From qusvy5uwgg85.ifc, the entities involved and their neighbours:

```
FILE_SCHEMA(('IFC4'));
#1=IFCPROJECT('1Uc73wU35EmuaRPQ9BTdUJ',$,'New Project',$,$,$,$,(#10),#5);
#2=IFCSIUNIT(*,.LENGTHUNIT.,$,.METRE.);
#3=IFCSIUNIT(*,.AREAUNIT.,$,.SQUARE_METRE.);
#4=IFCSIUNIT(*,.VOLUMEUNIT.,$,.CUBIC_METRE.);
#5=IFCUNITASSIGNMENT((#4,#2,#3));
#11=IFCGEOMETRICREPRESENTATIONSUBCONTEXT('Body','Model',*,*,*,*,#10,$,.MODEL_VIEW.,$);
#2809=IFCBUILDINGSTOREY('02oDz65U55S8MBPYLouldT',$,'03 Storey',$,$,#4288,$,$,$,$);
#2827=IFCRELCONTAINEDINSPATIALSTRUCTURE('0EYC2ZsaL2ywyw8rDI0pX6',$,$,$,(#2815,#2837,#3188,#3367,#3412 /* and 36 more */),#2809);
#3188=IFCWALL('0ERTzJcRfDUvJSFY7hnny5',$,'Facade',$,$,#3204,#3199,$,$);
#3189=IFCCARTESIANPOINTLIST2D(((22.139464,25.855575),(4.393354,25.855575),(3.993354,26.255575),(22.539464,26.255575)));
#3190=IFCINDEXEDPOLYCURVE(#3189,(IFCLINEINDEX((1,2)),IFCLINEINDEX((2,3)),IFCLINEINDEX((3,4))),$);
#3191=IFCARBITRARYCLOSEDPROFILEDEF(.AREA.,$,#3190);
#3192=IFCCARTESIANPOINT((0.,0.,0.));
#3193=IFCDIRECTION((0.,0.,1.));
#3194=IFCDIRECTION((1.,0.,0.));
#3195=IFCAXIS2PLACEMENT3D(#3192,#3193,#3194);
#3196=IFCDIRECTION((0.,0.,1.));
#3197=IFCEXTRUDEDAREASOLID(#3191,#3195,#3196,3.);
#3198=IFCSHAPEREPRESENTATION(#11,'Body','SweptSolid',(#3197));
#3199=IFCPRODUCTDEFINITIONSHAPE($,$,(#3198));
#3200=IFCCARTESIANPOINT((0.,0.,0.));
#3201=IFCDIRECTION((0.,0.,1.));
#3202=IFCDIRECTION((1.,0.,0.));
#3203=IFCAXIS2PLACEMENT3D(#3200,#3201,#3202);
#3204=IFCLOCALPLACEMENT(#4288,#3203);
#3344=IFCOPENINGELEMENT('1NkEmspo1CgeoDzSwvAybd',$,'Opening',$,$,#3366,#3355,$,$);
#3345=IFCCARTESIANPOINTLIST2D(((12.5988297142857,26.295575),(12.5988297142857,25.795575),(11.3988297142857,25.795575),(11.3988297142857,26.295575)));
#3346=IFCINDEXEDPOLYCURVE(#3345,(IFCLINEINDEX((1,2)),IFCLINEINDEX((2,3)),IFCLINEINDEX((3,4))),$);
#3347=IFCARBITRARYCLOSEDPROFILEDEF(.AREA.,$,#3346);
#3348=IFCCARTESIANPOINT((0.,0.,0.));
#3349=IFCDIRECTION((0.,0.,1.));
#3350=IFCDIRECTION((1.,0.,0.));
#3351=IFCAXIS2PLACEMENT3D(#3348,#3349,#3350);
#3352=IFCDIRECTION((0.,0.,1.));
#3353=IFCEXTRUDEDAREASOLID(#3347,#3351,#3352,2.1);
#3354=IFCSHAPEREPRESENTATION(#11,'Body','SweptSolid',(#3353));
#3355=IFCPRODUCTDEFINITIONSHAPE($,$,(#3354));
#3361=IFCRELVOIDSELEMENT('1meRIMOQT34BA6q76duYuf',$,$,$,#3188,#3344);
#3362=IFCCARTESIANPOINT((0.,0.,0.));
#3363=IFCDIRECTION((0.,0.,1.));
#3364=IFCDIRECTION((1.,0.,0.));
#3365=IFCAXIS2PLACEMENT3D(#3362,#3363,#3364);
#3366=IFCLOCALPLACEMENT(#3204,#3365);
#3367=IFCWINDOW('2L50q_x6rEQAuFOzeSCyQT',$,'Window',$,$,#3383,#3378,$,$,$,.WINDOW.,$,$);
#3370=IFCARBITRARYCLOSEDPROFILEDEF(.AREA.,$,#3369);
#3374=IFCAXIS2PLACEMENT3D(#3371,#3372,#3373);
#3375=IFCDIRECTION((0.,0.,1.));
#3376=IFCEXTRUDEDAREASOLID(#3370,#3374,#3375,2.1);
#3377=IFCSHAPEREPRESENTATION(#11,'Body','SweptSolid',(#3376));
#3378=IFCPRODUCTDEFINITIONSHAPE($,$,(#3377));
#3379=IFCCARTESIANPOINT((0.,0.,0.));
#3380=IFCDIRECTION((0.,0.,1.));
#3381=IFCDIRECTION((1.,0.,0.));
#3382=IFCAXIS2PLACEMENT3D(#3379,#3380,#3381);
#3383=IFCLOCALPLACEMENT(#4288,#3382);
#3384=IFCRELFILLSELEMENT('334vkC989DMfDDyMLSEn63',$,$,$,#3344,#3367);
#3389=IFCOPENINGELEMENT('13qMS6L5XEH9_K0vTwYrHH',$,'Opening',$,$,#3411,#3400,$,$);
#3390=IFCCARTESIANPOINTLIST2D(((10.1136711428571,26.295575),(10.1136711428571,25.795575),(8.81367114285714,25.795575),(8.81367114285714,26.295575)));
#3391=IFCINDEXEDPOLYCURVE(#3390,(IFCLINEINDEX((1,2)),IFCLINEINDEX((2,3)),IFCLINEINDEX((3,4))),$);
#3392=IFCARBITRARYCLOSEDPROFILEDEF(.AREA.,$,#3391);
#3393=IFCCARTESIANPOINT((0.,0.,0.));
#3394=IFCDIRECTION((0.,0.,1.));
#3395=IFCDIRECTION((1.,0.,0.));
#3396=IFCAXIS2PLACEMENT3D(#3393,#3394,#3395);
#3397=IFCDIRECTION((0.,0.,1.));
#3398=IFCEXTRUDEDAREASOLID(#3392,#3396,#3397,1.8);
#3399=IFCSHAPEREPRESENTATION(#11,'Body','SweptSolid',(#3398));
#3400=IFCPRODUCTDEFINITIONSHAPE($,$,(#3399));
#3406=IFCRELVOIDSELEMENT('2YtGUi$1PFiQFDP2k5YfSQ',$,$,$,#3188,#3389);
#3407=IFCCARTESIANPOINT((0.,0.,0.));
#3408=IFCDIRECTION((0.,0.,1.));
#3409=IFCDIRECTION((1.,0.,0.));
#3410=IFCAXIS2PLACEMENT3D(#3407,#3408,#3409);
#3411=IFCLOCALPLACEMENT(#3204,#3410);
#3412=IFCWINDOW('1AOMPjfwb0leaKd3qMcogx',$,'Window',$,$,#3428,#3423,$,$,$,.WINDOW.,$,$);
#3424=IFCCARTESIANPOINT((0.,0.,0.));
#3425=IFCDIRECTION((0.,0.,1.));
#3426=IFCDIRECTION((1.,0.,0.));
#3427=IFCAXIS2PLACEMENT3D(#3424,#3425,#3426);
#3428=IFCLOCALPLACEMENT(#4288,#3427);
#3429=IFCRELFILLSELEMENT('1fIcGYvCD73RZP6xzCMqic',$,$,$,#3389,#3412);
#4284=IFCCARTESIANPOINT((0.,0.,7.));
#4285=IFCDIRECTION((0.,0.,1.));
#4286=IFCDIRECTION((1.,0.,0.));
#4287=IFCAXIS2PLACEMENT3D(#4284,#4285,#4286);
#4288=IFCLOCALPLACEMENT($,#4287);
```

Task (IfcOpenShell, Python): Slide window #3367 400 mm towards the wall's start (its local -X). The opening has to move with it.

```python
import ifcopenshell
import ifcopenshell.api.geometry
import ifcopenshell.util.placement
import ifcopenshell.util.unit

model = ifcopenshell.open("qusvy5uwgg85.ifc")
unit_scale = ifcopenshell.util.unit.calculate_unit_scale(model)

window = model.by_guid("2L50q_x6rEQAuFOzeSCyQT")
opening = window.FillsVoids[0].RelatingOpeningElement
wall = opening.VoidsElements[0].RelatingBuildingElement

wall_matrix = ifcopenshell.util.placement.get_local_placement(wall.ObjectPlacement)
shift = wall_matrix[:3, 0] * -0.4 / unit_scale
before = ifcopenshell.util.placement.get_local_placement(window.ObjectPlacement)[:3, 3].copy()

# The window is not placed relative to its opening, so move both.
for product in (opening, window):
    matrix = ifcopenshell.util.placement.get_local_placement(product.ObjectPlacement)
    matrix[:3, 3] += shift
    ifcopenshell.api.geometry.edit_object_placement(model, product=product, matrix=matrix, is_si=False)

after = ifcopenshell.util.placement.get_local_placement(window.ObjectPlacement)[:3, 3]
print("window moved by", (after - before).round(3) + 0.0)

model.write("qusvy5uwgg85_rev.ifc")
```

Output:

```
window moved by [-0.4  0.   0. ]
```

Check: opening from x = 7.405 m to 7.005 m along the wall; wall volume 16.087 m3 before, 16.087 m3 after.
